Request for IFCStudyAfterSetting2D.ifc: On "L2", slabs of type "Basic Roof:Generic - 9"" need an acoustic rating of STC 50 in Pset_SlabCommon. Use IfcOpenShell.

First a look at what the model holds.

```python
import ifcopenshell
import ifcopenshell.util.element

model = ifcopenshell.open("IFCStudyAfterSetting2D.ifc")
print(model.schema)
storey = next(s for s in model.by_type("IfcBuildingStorey") if s.Name == "L2")
slabs = [e for e in ifcopenshell.util.element.get_decomposition(storey) if e.is_a("IfcSlab")]
seen = {}
for e in slabs:
    element_type = ifcopenshell.util.element.get_type(e)
    key = (element_type.Name if element_type != e and element_type else None, ifcopenshell.util.element.get_pset(e, "Pset_SlabCommon", "AcousticRating"))
    seen[key] = seen.get(key, 0) + 1
for (name, value), count in sorted(seen.items(), key=str):
    print(count, "x", name, "|", value)
```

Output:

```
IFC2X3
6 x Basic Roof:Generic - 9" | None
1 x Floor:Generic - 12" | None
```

```python
import ifcopenshell
import ifcopenshell.api.pset
import ifcopenshell.util.element

model = ifcopenshell.open("IFCStudyAfterSetting2D.ifc")

storey = next(s for s in model.by_type("IfcBuildingStorey") if s.Name == "L2")
slabs = [e for e in ifcopenshell.util.element.get_decomposition(storey) if e.is_a("IfcSlab")]

count = 0
for e in slabs:
    element_type = ifcopenshell.util.element.get_type(e)
    if element_type in (None, e) or element_type.Name != 'Basic Roof:Generic - 9"':
        continue
    # add_pset returns the element's existing set when there is one.
    pset = ifcopenshell.api.pset.add_pset(model, product=e, name="Pset_SlabCommon")
    ifcopenshell.api.pset.edit_pset(model, pset=pset, properties={"AcousticRating": "STC 50"})
    count += 1

print(count, "slabs updated")

model.write("IFCStudyAfterSetting2D_updated.ifc")
```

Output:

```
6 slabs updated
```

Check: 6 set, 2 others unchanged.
